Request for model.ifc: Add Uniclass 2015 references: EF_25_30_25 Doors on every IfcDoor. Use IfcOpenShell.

First a look at what the model holds.

```python
import ifcopenshell

model = ifcopenshell.open("model.ifc")
print(model.schema)
print("classifications:", [c.Name for c in model.by_type("IfcClassification")])
for ifc_class in ("IfcDoor", "IfcRoof", "IfcStair", "IfcWall", "IfcWindow"):
    print(ifc_class, len(model.by_type(ifc_class)))
```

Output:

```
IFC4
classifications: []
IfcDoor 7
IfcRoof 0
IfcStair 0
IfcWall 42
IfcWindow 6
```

```python
import ifcopenshell
import ifcopenshell.api.classification

model = ifcopenshell.open("model.ifc")

system = ifcopenshell.api.classification.add_classification(model, classification="Uniclass 2015")

codes = {
    "IfcDoor": ("EF_25_30_25", "Doors"),
}
for ifc_class, (code, name) in codes.items():
    products = model.by_type(ifc_class)
    ifcopenshell.api.classification.add_reference(
        model, products=products, classification=system, identification=code, name=name
    )
    print(code, len(products))

model.write("model_rev.ifc")
```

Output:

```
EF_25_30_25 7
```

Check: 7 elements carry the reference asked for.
